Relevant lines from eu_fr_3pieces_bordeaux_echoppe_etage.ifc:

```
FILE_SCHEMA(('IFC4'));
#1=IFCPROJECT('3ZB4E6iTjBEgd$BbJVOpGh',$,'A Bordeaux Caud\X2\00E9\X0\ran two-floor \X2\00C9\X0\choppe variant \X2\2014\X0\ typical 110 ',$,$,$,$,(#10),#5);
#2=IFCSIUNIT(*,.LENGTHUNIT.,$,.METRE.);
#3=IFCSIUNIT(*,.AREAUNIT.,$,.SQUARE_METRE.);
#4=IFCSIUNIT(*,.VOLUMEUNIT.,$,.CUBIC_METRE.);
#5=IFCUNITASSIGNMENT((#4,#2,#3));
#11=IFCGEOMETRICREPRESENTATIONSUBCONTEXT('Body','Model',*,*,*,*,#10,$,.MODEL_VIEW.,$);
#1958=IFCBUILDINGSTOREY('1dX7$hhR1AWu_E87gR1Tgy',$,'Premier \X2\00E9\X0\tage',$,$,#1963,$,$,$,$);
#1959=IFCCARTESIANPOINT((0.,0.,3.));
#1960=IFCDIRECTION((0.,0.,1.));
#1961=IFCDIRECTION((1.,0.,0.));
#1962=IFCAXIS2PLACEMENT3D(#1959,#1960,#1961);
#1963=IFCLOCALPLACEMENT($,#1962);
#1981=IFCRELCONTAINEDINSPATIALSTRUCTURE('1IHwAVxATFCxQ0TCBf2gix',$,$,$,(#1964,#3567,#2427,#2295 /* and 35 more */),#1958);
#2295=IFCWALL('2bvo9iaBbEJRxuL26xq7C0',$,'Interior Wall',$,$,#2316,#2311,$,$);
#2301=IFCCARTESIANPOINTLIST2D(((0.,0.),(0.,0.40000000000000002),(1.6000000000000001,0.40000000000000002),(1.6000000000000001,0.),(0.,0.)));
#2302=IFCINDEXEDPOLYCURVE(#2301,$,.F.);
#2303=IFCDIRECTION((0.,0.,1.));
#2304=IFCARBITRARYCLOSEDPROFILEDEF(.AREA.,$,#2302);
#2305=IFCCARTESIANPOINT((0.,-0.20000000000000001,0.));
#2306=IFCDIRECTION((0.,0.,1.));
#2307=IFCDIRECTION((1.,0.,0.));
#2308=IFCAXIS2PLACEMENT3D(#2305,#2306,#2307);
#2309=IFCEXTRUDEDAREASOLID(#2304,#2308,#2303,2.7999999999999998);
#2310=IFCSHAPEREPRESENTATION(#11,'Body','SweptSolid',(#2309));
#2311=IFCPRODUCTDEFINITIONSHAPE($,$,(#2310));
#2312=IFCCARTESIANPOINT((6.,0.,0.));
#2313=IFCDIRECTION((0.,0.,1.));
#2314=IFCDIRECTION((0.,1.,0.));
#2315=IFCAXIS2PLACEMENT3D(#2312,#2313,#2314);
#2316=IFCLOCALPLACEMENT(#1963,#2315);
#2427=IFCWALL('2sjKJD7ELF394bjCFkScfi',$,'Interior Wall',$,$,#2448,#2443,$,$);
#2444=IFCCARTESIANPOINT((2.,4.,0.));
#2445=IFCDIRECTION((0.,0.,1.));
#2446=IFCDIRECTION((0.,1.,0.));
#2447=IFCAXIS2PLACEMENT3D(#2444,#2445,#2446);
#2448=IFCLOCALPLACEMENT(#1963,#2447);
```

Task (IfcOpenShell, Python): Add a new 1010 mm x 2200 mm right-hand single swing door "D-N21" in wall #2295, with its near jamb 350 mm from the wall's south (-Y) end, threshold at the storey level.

```python
import numpy as np
import ifcopenshell
import ifcopenshell.api.feature
import ifcopenshell.api.geometry
import ifcopenshell.api.root
import ifcopenshell.api.spatial
import ifcopenshell.geom
import ifcopenshell.util.element
import ifcopenshell.util.placement
import ifcopenshell.util.representation
import ifcopenshell.util.shape
import ifcopenshell.util.unit

model = ifcopenshell.open("eu_fr_3pieces_bordeaux_echoppe_etage.ifc")
unit_scale = ifcopenshell.util.unit.calculate_unit_scale(model)
settings = ifcopenshell.geom.settings()


def volume(element):
    """Net volume in cubic metres, openings subtracted."""
    shape = ifcopenshell.geom.create_shape(settings, element)
    return ifcopenshell.util.shape.get_volume(shape.geometry)


wall = model.by_guid("2bvo9iaBbEJRxuL26xq7C0")
storey = ifcopenshell.util.element.get_container(wall, ifc_class="IfcBuildingStorey")
context = ifcopenshell.util.representation.get_context(model, "Model", "Body", "MODEL_VIEW")
before = volume(wall)

width, height, from_end, sill = 1.01, 2.2, 0.35, 0.0  # metres

# The wall runs along its own X axis, and the end named is its -X end.
wall_shape = ifcopenshell.geom.create_shape(settings, wall)
x, y, z = ifcopenshell.util.shape.get_vertices(wall_shape.geometry).T
start = x.min() + from_end
face, thickness = float(y.min()), float(y.max() - y.min())
wall_matrix = ifcopenshell.util.placement.get_local_placement(wall.ObjectPlacement)
level = ifcopenshell.util.placement.get_local_placement(storey.ObjectPlacement)[2, 3]


def in_wall(x, y):
    """Placement at x, y metres in the wall's axes, at sill height."""
    matrix = wall_matrix.copy()
    matrix[:, 3] = wall_matrix @ np.array([x / unit_scale, y / unit_scale, 0.0, 1.0])
    matrix[2, 3] = level + sill / unit_scale
    return matrix


# Opening: a box that overshoots both wall faces by 50 mm.
opening = ifcopenshell.api.root.create_entity(model, ifc_class="IfcOpeningElement", predefined_type="OPENING")
box = ifcopenshell.api.geometry.add_wall_representation(
    model, context=context, length=width, height=height, thickness=thickness + 0.1
)
ifcopenshell.api.geometry.assign_representation(model, product=opening, representation=box)
ifcopenshell.api.geometry.edit_object_placement(model, product=opening, matrix=in_wall(start, face - 0.05), is_si=False)
ifcopenshell.api.feature.add_feature(model, feature=opening, element=wall)

door = ifcopenshell.api.root.create_entity(model, ifc_class="IfcDoor", name="D-N21", predefined_type="DOOR")
door.OverallWidth, door.OverallHeight = width / unit_scale, height / unit_scale
door.OperationType = "SINGLE_SWING_RIGHT"
body = ifcopenshell.api.geometry.add_door_representation(
    model,
    context=context,
    overall_width=door.OverallWidth,
    overall_height=door.OverallHeight,
    operation_type="SINGLE_SWING_RIGHT",
    lining_properties={"LiningDepth": thickness / unit_scale, "ThresholdDepth": thickness / unit_scale},
)
ifcopenshell.api.geometry.assign_representation(model, product=door, representation=body)
ifcopenshell.api.spatial.assign_container(model, products=[door], relating_structure=storey)
ifcopenshell.api.feature.add_filling(model, opening=opening, element=door)

# The lining spans the wall, so the door starts at the wall face.
ifcopenshell.api.geometry.edit_object_placement(model, product=door, matrix=in_wall(start, face), is_si=False)

after = volume(wall)

print(f"wall volume {before:.3f} -> {after:.3f} m3")

model.write("eu_fr_3pieces_bordeaux_echoppe_etage-out.ifc")
```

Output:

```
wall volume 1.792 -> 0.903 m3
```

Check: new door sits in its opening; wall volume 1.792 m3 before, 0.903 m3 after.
